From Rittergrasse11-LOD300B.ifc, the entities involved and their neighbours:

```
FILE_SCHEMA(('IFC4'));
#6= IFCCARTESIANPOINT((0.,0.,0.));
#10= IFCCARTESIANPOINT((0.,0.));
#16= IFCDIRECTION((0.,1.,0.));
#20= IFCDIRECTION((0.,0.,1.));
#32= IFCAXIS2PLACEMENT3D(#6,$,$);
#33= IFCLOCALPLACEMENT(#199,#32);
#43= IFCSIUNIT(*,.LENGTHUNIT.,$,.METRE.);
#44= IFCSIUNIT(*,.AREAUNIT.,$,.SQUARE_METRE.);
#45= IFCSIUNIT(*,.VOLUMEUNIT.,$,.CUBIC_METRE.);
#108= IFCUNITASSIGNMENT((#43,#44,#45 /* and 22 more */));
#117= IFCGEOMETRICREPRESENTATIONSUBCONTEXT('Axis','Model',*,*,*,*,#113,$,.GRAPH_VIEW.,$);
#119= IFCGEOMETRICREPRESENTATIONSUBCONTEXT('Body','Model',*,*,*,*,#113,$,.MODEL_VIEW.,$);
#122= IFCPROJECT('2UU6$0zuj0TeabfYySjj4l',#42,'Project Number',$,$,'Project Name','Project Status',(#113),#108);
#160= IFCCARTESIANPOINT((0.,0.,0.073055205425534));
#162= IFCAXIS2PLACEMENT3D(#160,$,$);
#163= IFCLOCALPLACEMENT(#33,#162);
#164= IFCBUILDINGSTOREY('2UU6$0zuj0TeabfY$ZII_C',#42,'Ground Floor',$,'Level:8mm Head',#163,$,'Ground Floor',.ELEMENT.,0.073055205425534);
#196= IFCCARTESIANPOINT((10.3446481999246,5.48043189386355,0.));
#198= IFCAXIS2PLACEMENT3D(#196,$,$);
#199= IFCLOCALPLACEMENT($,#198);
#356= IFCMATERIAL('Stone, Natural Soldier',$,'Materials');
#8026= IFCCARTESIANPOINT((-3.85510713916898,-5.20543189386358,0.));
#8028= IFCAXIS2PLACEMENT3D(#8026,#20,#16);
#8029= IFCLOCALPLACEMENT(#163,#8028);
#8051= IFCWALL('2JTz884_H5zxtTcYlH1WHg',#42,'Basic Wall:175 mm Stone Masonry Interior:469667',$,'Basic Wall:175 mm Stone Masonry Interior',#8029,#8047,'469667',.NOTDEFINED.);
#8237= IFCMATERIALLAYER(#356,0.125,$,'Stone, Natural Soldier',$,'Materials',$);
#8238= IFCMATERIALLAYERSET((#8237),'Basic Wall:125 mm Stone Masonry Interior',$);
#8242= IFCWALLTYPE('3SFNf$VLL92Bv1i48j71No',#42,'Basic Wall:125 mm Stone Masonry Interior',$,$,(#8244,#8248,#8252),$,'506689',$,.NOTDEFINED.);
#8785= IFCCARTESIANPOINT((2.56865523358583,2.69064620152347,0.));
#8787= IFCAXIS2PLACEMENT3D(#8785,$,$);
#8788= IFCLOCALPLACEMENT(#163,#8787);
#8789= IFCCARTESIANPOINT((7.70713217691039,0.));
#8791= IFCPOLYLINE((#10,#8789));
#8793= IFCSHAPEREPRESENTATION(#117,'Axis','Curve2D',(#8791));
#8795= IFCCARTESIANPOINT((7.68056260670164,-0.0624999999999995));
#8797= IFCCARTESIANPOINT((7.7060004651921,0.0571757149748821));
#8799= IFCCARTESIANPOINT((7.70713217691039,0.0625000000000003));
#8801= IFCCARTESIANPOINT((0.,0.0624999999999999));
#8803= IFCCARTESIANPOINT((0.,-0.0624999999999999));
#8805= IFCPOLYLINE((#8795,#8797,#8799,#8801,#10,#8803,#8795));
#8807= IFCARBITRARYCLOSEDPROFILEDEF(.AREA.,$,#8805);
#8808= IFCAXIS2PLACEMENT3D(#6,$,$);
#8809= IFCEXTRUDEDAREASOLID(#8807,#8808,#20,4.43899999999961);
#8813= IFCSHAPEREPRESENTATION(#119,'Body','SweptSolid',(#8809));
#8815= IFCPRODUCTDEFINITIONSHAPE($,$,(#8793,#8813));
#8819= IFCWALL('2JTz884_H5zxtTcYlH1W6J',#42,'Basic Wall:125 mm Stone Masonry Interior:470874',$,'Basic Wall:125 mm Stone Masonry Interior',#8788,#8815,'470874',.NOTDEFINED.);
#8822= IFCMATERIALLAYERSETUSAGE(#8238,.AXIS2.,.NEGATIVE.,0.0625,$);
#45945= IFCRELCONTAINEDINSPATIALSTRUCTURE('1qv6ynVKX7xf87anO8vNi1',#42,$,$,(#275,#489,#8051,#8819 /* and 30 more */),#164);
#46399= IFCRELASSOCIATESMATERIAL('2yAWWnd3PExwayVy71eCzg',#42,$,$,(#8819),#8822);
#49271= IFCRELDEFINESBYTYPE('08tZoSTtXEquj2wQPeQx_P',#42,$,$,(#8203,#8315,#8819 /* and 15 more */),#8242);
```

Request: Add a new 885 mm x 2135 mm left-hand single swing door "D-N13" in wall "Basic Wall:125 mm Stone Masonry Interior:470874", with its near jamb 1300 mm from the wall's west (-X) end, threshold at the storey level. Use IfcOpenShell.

```python
import numpy as np
import ifcopenshell
import ifcopenshell.api.feature
import ifcopenshell.api.geometry
import ifcopenshell.api.root
import ifcopenshell.api.spatial
import ifcopenshell.geom
import ifcopenshell.util.element
import ifcopenshell.util.placement
import ifcopenshell.util.representation
import ifcopenshell.util.shape
import ifcopenshell.util.unit

model = ifcopenshell.open("Rittergrasse11-LOD300B.ifc")
unit_scale = ifcopenshell.util.unit.calculate_unit_scale(model)
settings = ifcopenshell.geom.settings()


def volume(element):
    """Net volume in cubic metres, openings subtracted."""
    shape = ifcopenshell.geom.create_shape(settings, element)
    return ifcopenshell.util.shape.get_volume(shape.geometry)


wall = model.by_guid("2JTz884_H5zxtTcYlH1W6J")
storey = ifcopenshell.util.element.get_container(wall, ifc_class="IfcBuildingStorey")
context = ifcopenshell.util.representation.get_context(model, "Model", "Body", "MODEL_VIEW")
before = volume(wall)

width, height, from_end, sill = 0.885, 2.135, 1.3, 0.0  # metres

# The wall runs along its own X axis, and the end named is its -X end.
wall_shape = ifcopenshell.geom.create_shape(settings, wall)
x, y, z = ifcopenshell.util.shape.get_vertices(wall_shape.geometry).T
start = x.min() + from_end
face, thickness = float(y.min()), float(y.max() - y.min())
wall_matrix = ifcopenshell.util.placement.get_local_placement(wall.ObjectPlacement)
level = ifcopenshell.util.placement.get_local_placement(storey.ObjectPlacement)[2, 3]


def in_wall(x, y):
    """Placement at x, y metres in the wall's axes, at sill height."""
    matrix = wall_matrix.copy()
    matrix[:, 3] = wall_matrix @ np.array([x / unit_scale, y / unit_scale, 0.0, 1.0])
    matrix[2, 3] = level + sill / unit_scale
    return matrix


# Opening: a box that overshoots both wall faces by 50 mm.
opening = ifcopenshell.api.root.create_entity(model, ifc_class="IfcOpeningElement", predefined_type="OPENING")
box = ifcopenshell.api.geometry.add_wall_representation(
    model, context=context, length=width, height=height, thickness=thickness + 0.1
)
ifcopenshell.api.geometry.assign_representation(model, product=opening, representation=box)
ifcopenshell.api.geometry.edit_object_placement(model, product=opening, matrix=in_wall(start, face - 0.05), is_si=False)
ifcopenshell.api.feature.add_feature(model, feature=opening, element=wall)

door = ifcopenshell.api.root.create_entity(model, ifc_class="IfcDoor", name="D-N13", predefined_type="DOOR")
door.OverallWidth, door.OverallHeight = width / unit_scale, height / unit_scale
door.OperationType = "SINGLE_SWING_LEFT"
body = ifcopenshell.api.geometry.add_door_representation(
    model,
    context=context,
    overall_width=door.OverallWidth,
    overall_height=door.OverallHeight,
    operation_type="SINGLE_SWING_LEFT",
    lining_properties={"LiningDepth": thickness / unit_scale, "ThresholdDepth": thickness / unit_scale},
)
ifcopenshell.api.geometry.assign_representation(model, product=door, representation=body)
ifcopenshell.api.spatial.assign_container(model, products=[door], relating_structure=storey)
ifcopenshell.api.feature.add_filling(model, opening=opening, element=door)

# The lining spans the wall, so the door starts at the wall face.
ifcopenshell.api.geometry.edit_object_placement(model, product=door, matrix=in_wall(start, face), is_si=False)

after = volume(wall)

print(f"wall volume {before:.3f} -> {after:.3f} m3")

model.write("Rittergrasse11-LOD300B-out.ifc")
```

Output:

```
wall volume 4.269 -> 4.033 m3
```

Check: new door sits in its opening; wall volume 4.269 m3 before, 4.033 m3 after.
